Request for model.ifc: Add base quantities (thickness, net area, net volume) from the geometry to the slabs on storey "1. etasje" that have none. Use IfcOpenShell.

First a look at what the model holds.

```python
import ifcopenshell
import ifcopenshell.util.element
import ifcopenshell.util.unit

model = ifcopenshell.open("model.ifc")
print(model.schema)
for unit_type in ("LENGTHUNIT", "AREAUNIT", "VOLUMEUNIT"):
    print(unit_type, ifcopenshell.util.unit.calculate_unit_scale(model, unit_type))
storey = next(s for s in model.by_type("IfcBuildingStorey") if s.Name == "1. etasje")
slabs = [e for e in ifcopenshell.util.element.get_decomposition(storey) if e.is_a("IfcSlab")]
for e in sorted(slabs, key=lambda e: e.id()):
    print(e.id(), e.is_a(), e.Name, list(ifcopenshell.util.element.get_psets(e, qtos_only=True)), sep=" | ")
```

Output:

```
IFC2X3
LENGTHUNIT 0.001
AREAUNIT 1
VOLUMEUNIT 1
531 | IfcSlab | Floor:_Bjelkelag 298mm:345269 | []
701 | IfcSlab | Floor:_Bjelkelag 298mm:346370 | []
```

```python
import ifcopenshell
import ifcopenshell.api.pset
import ifcopenshell.geom
import ifcopenshell.util.element
import ifcopenshell.util.shape
import ifcopenshell.util.unit

model = ifcopenshell.open("model.ifc")
unit_scale = ifcopenshell.util.unit.calculate_unit_scale(model)
area_scale = ifcopenshell.util.unit.calculate_unit_scale(model, "AREAUNIT")
volume_scale = ifcopenshell.util.unit.calculate_unit_scale(model, "VOLUMEUNIT")
settings = ifcopenshell.geom.settings()

storey = next(s for s in model.by_type("IfcBuildingStorey") if s.Name == "1. etasje")
slabs = [e for e in ifcopenshell.util.element.get_decomposition(storey) if e.is_a("IfcSlab")]

for e in sorted(slabs, key=lambda e: e.id()):
    if ifcopenshell.util.element.get_psets(e, qtos_only=True, should_inherit=False):
        continue
    # Geometry comes back in metres, in the element's own axes.
    shape = ifcopenshell.geom.create_shape(settings, e)
    values = {
        "Width": ifcopenshell.util.shape.get_z(shape.geometry) / unit_scale,
        "NetArea": ifcopenshell.util.shape.get_footprint_area(shape.geometry) / area_scale,
        "NetVolume": ifcopenshell.util.shape.get_volume(shape.geometry) / volume_scale,
    }
    qto = ifcopenshell.api.pset.add_qto(model, product=e, name="BaseQuantities")
    ifcopenshell.api.pset.edit_qto(model, qto=qto, properties=values)
    print(e.id(), {k: round(v, 3) for k, v in values.items()})

model.write("model_rev.ifc")
```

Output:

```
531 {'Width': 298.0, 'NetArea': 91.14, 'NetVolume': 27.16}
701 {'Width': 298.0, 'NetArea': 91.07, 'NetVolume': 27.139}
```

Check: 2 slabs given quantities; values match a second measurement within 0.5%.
